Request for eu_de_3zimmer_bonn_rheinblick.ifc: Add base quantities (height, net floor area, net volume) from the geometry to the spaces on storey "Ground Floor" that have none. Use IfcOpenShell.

First a look at what the model holds.

```python
import ifcopenshell
import ifcopenshell.util.element
import ifcopenshell.util.unit

model = ifcopenshell.open("eu_de_3zimmer_bonn_rheinblick.ifc")
print(model.schema)
for unit_type in ("LENGTHUNIT", "AREAUNIT", "VOLUMEUNIT"):
    print(unit_type, ifcopenshell.util.unit.calculate_unit_scale(model, unit_type))
storey = next(s for s in model.by_type("IfcBuildingStorey") if s.Name == "Ground Floor")
spaces = [e for e in ifcopenshell.util.element.get_decomposition(storey) if e.is_a("IfcSpace")]
for e in sorted(spaces, key=lambda e: e.id()):
    print(e.id(), e.is_a(), e.Name, list(ifcopenshell.util.element.get_psets(e, qtos_only=True)), sep=" | ")
```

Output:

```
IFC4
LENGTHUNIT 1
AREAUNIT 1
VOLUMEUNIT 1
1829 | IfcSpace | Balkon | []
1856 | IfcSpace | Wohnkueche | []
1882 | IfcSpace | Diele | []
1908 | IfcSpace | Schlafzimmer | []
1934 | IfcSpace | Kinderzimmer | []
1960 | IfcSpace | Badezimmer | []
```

```python
import ifcopenshell
import ifcopenshell.api.pset
import ifcopenshell.geom
import ifcopenshell.util.element
import ifcopenshell.util.shape
import ifcopenshell.util.unit

model = ifcopenshell.open("eu_de_3zimmer_bonn_rheinblick.ifc")
unit_scale = ifcopenshell.util.unit.calculate_unit_scale(model)
area_scale = ifcopenshell.util.unit.calculate_unit_scale(model, "AREAUNIT")
volume_scale = ifcopenshell.util.unit.calculate_unit_scale(model, "VOLUMEUNIT")
settings = ifcopenshell.geom.settings()

storey = next(s for s in model.by_type("IfcBuildingStorey") if s.Name == "Ground Floor")
spaces = [e for e in ifcopenshell.util.element.get_decomposition(storey) if e.is_a("IfcSpace")]

for e in sorted(spaces, key=lambda e: e.id()):
    if ifcopenshell.util.element.get_psets(e, qtos_only=True, should_inherit=False):
        continue
    # Geometry comes back in metres, in the element's own axes.
    shape = ifcopenshell.geom.create_shape(settings, e)
    values = {
        "Height": ifcopenshell.util.shape.get_z(shape.geometry) / unit_scale,
        "NetFloorArea": ifcopenshell.util.shape.get_footprint_area(shape.geometry) / area_scale,
        "NetVolume": ifcopenshell.util.shape.get_volume(shape.geometry) / volume_scale,
    }
    qto = ifcopenshell.api.pset.add_qto(model, product=e, name="Qto_SpaceBaseQuantities")
    ifcopenshell.api.pset.edit_qto(model, qto=qto, properties=values)
    print(e.id(), {k: round(v, 3) for k, v in values.items()})

model.write("eu_de_3zimmer_bonn_rheinblick_v2.ifc")
```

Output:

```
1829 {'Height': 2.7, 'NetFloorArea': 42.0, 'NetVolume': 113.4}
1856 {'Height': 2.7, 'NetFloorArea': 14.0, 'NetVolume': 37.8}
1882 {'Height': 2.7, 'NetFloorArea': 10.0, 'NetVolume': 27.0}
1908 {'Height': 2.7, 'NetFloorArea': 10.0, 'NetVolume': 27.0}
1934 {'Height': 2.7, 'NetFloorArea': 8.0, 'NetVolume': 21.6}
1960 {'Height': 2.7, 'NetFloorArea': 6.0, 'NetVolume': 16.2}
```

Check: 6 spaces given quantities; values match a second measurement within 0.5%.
